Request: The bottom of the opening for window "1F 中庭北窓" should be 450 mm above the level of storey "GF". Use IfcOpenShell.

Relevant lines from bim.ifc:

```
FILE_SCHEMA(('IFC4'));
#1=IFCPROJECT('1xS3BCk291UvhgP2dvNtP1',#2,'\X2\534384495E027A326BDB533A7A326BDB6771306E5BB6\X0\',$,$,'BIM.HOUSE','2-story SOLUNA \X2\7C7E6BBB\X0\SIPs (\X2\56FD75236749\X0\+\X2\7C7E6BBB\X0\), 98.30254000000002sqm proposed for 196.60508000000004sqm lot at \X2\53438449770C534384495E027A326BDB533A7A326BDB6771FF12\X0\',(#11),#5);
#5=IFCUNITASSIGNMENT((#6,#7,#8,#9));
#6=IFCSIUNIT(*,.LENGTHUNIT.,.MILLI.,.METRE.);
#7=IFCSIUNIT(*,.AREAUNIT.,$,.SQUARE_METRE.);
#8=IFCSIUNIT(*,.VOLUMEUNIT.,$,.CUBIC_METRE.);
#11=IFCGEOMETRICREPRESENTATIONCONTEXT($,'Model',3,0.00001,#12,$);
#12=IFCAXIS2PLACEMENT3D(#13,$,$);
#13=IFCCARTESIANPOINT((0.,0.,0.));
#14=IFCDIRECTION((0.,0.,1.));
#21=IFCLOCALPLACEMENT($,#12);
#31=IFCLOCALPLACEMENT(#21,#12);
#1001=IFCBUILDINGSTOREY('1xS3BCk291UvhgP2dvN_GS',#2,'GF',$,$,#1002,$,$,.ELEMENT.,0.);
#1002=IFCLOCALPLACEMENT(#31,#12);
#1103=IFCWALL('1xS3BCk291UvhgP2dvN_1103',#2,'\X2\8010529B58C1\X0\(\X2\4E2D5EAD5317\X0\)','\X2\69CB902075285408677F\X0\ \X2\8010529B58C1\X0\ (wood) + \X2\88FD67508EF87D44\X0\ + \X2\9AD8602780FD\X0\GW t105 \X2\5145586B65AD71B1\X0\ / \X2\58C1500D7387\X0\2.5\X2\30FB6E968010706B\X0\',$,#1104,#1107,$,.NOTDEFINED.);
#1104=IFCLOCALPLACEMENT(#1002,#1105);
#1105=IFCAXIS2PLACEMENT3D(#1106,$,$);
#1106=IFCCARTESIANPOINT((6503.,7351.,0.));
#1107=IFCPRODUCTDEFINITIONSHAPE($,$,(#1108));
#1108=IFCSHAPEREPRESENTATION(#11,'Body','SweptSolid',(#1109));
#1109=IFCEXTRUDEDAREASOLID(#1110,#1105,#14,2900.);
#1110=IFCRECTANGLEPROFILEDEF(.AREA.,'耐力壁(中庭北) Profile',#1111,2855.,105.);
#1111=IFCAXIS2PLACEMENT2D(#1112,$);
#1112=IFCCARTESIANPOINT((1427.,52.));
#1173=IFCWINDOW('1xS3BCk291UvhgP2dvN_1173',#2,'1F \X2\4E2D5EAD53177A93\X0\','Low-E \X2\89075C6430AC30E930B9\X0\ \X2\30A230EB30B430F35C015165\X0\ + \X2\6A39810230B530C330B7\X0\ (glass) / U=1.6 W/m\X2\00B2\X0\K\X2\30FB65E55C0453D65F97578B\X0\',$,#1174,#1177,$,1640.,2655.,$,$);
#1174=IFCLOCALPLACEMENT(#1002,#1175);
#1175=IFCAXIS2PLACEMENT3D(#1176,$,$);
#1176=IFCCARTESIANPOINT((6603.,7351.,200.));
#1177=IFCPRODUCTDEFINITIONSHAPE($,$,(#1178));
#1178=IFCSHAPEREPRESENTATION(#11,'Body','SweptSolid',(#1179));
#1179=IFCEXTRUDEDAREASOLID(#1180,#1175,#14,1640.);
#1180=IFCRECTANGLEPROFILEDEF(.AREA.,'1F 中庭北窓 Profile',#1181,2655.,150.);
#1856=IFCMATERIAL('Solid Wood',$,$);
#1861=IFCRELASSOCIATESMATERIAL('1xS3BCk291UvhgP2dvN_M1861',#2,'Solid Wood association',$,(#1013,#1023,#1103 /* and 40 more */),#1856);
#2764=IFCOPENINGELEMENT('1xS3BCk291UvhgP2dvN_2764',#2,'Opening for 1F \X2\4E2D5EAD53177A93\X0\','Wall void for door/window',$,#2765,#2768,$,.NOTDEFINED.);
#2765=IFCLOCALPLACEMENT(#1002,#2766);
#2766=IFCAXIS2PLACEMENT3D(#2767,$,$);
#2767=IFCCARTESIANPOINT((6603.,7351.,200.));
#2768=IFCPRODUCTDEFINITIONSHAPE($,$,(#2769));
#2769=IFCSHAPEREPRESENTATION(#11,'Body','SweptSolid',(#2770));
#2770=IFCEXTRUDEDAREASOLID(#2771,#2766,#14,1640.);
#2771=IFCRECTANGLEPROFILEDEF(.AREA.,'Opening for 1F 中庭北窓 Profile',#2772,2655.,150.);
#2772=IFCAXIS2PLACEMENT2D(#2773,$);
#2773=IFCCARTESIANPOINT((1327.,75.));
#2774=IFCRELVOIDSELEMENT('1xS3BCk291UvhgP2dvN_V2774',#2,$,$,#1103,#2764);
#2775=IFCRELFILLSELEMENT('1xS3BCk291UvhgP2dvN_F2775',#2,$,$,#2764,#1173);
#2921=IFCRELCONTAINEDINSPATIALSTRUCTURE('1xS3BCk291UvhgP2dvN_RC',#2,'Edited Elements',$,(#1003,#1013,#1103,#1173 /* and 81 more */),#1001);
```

```python
import numpy as np
import ifcopenshell
import ifcopenshell.api.geometry
import ifcopenshell.geom
import ifcopenshell.util.element
import ifcopenshell.util.placement
import ifcopenshell.util.shape
import ifcopenshell.util.unit

model = ifcopenshell.open("bim.ifc")
unit_scale = ifcopenshell.util.unit.calculate_unit_scale(model)

window = model.by_id(1173)
opening = window.FillsVoids[0].RelatingOpeningElement
storey = ifcopenshell.util.element.get_container(window, ifc_class="IfcBuildingStorey")
level = ifcopenshell.util.placement.get_local_placement(storey.ObjectPlacement)[2, 3]

# The opening's origin need not be at the sill, so measure its lowest point.
shape = ifcopenshell.geom.create_shape(ifcopenshell.geom.settings(), opening)
bottom = ifcopenshell.util.shape.get_shape_bottom_elevation(shape, shape.geometry) / unit_scale
dz = level + 0.45 / unit_scale - bottom

shift = np.array([0.0, 0.0, dz])
# The window is not placed relative to its opening, so move both.
for product in (opening, window):
    matrix = ifcopenshell.util.placement.get_local_placement(product.ObjectPlacement)
    matrix[:3, 3] += shift
    ifcopenshell.api.geometry.edit_object_placement(model, product=product, matrix=matrix, is_si=False)

print(f"moved by {dz * unit_scale:+.3f} m")

model.write("bim_v2.ifc")
```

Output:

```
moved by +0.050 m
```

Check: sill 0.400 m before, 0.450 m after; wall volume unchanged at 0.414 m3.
